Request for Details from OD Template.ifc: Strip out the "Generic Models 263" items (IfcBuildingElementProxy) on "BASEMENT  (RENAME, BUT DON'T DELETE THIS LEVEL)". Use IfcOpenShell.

First a look at what the model holds.

```python
import ifcopenshell
import ifcopenshell.util.element

model = ifcopenshell.open("Details from OD Template.ifc")
print(model.schema)
storey = next(s for s in model.by_type("IfcBuildingStorey") if s.Name == "BASEMENT  (RENAME, BUT DON'T DELETE THIS LEVEL)")
proxies = [e for e in ifcopenshell.util.element.get_decomposition(storey) if e.is_a("IfcBuildingElementProxy")]
seen = {}
for e in proxies:
    element_type = ifcopenshell.util.element.get_type(e)
    name = element_type.Name if element_type not in (None, e) else None
    seen[name] = seen.get(name, 0) + 1
for name, count in sorted(seen.items(), key=str):
    print(count, "x", name)
```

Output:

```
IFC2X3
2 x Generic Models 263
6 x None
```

```python
import ifcopenshell
import ifcopenshell.api.root
import ifcopenshell.util.element

model = ifcopenshell.open("Details from OD Template.ifc")

storey = next(s for s in model.by_type("IfcBuildingStorey") if s.Name == "BASEMENT  (RENAME, BUT DON'T DELETE THIS LEVEL)")
proxies = [e for e in ifcopenshell.util.element.get_decomposition(storey) if e.is_a("IfcBuildingElementProxy")]
targets = [e for e in proxies if (t := ifcopenshell.util.element.get_type(e)) not in (None, e) and t.Name == "Generic Models 263"]

for e in targets:
    ifcopenshell.api.root.remove_product(model, product=e)
print(len(targets), "removed")

model.write("Details from OD Template_updated.ifc")
```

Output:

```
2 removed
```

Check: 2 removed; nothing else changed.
